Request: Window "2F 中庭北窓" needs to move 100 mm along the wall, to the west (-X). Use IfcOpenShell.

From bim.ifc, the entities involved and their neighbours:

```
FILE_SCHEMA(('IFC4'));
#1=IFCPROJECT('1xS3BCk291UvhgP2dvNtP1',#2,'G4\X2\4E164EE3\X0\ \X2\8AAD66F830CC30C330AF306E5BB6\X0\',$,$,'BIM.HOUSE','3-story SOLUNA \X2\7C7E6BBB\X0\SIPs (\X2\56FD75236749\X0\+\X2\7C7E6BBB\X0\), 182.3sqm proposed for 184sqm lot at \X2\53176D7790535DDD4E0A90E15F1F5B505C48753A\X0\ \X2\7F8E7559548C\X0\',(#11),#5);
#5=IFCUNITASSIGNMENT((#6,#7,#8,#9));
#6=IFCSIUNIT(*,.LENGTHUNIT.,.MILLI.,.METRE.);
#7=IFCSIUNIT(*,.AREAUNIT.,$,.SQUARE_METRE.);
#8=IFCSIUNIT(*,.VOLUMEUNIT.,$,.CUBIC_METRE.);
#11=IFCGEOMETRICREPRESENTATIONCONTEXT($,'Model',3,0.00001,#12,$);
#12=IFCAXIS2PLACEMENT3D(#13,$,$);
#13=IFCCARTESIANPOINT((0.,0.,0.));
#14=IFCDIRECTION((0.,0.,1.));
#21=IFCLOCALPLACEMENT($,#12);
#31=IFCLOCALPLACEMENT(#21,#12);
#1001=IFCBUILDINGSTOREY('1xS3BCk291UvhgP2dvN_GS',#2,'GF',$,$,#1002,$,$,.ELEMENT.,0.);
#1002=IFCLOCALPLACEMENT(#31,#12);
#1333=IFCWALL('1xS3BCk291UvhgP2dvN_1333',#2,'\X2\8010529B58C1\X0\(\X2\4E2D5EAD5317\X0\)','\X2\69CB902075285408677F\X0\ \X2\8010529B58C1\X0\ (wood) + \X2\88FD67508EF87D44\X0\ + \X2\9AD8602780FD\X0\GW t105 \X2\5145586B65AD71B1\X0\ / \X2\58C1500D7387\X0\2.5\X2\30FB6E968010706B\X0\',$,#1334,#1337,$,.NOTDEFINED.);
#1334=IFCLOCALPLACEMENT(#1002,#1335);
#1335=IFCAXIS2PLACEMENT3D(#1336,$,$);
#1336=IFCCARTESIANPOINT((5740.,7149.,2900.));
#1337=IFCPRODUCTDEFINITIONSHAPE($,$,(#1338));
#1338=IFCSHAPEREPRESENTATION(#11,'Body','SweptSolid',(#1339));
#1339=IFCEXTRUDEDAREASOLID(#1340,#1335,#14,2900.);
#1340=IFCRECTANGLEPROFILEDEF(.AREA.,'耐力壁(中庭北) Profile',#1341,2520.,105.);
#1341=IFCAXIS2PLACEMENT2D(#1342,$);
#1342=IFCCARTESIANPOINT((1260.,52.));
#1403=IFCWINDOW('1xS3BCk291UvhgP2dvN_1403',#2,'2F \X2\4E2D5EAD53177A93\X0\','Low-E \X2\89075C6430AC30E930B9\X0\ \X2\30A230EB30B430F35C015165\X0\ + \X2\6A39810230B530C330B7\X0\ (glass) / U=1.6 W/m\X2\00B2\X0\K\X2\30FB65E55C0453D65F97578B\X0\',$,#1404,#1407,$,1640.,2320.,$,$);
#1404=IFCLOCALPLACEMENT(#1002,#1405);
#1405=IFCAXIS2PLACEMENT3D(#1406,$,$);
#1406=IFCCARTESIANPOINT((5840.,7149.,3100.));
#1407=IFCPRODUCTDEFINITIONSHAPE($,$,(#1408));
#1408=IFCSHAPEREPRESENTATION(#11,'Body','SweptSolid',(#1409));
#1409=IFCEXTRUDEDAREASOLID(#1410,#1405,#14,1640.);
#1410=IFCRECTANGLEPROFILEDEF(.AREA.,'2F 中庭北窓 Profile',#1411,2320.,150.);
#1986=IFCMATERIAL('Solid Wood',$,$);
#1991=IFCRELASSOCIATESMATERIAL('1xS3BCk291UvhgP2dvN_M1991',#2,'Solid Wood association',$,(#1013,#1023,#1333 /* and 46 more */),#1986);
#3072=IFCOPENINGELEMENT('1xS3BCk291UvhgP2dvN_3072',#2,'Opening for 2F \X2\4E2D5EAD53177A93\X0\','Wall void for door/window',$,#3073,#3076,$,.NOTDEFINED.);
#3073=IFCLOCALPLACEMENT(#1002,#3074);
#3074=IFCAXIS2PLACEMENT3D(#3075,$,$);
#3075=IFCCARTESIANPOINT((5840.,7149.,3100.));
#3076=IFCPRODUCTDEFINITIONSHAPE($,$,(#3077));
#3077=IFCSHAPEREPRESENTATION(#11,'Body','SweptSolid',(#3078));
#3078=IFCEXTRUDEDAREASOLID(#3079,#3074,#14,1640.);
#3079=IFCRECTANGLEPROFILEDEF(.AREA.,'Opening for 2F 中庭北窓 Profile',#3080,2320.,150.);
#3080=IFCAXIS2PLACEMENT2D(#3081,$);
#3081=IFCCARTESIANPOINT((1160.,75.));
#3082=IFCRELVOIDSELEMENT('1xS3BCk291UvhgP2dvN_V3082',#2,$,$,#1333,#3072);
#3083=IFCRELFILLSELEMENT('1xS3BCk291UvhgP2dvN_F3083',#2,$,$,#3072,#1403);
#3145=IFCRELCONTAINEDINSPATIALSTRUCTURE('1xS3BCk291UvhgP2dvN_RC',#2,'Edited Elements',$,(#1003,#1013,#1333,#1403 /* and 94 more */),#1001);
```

```python
import ifcopenshell
import ifcopenshell.api.geometry
import ifcopenshell.util.placement
import ifcopenshell.util.unit

model = ifcopenshell.open("bim.ifc")
unit_scale = ifcopenshell.util.unit.calculate_unit_scale(model)

window = model.by_id(1403)
opening = window.FillsVoids[0].RelatingOpeningElement
wall = opening.VoidsElements[0].RelatingBuildingElement

wall_matrix = ifcopenshell.util.placement.get_local_placement(wall.ObjectPlacement)
shift = wall_matrix[:3, 0] * -0.1 / unit_scale
before = ifcopenshell.util.placement.get_local_placement(window.ObjectPlacement)[:3, 3].copy()

# The window is not placed relative to its opening, so move both.
for product in (opening, window):
    matrix = ifcopenshell.util.placement.get_local_placement(product.ObjectPlacement)
    matrix[:3, 3] += shift
    ifcopenshell.api.geometry.edit_object_placement(model, product=product, matrix=matrix, is_si=False)

after = ifcopenshell.util.placement.get_local_placement(window.ObjectPlacement)[:3, 3]
print("window moved by", (after - before).round(3) + 0.0)

model.write("bim_rev.ifc")
```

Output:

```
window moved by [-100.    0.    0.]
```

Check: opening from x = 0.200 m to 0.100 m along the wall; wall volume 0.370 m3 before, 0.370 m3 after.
